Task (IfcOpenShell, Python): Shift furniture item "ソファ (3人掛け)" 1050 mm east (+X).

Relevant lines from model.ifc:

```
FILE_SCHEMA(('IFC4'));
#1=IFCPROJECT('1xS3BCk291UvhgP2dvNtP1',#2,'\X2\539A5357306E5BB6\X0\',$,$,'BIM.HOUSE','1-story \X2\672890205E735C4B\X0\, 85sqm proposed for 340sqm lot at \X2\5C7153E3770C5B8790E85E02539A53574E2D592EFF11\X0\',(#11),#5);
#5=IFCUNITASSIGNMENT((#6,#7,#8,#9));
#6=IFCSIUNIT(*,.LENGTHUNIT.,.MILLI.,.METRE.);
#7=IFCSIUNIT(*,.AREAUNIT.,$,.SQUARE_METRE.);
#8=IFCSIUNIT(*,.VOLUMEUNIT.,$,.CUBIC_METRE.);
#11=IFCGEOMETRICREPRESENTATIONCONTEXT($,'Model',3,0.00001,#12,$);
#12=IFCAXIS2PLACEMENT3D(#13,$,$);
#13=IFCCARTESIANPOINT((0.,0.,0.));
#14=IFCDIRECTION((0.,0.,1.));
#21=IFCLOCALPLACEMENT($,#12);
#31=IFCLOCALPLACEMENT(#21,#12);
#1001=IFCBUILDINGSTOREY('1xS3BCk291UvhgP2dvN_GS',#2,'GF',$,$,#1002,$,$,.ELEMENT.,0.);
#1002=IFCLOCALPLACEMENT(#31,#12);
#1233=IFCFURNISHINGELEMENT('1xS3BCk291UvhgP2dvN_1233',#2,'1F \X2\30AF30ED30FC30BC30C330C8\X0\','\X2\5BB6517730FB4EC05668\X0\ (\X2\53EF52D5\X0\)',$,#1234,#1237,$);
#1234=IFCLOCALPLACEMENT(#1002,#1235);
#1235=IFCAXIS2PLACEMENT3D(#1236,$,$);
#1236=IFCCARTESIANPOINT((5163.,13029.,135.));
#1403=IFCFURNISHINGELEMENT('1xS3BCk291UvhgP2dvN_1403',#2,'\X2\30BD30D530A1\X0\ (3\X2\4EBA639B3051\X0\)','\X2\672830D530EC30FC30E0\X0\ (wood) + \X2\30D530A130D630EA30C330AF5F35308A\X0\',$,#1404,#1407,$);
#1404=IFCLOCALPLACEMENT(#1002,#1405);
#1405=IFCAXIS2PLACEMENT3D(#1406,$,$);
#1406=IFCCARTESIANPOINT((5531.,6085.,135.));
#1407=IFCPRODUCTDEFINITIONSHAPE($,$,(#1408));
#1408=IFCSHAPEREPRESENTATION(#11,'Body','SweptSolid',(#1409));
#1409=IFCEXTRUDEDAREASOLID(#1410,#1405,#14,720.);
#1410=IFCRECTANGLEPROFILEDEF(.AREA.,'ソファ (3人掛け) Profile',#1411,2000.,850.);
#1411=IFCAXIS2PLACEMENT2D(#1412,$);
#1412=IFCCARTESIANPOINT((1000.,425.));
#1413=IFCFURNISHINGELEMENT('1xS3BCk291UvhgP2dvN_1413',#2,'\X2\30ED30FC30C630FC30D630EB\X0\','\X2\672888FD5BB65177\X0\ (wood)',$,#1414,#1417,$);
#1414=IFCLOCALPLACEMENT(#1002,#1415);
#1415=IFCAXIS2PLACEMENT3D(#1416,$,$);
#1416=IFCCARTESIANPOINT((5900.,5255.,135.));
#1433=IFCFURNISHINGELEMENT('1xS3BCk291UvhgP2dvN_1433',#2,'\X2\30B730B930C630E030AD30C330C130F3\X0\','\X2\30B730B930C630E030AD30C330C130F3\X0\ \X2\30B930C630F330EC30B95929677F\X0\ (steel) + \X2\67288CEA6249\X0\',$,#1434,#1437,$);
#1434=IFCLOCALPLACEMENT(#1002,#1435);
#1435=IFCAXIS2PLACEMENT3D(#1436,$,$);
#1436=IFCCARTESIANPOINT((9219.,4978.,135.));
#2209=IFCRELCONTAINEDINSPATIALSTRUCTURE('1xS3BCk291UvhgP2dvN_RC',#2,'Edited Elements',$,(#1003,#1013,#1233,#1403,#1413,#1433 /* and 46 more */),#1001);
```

```python
import ifcopenshell
import ifcopenshell.api.geometry
import ifcopenshell.util.placement
import ifcopenshell.util.unit

model = ifcopenshell.open("model.ifc")
unit_scale = ifcopenshell.util.unit.calculate_unit_scale(model)

item = model.by_guid("1xS3BCk291UvhgP2dvN_1403")
matrix = ifcopenshell.util.placement.get_local_placement(item.ObjectPlacement)
matrix[0, 3] += 1.05 / unit_scale
ifcopenshell.api.geometry.edit_object_placement(model, product=item, matrix=matrix, is_si=False)

print(ifcopenshell.util.placement.get_local_placement(item.ObjectPlacement).round(3) + 0.0)

model.write("model_edited.ifc")
```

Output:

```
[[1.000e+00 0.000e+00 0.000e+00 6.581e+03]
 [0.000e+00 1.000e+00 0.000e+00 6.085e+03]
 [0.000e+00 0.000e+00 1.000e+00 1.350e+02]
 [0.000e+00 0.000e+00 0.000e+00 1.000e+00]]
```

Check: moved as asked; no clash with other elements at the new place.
